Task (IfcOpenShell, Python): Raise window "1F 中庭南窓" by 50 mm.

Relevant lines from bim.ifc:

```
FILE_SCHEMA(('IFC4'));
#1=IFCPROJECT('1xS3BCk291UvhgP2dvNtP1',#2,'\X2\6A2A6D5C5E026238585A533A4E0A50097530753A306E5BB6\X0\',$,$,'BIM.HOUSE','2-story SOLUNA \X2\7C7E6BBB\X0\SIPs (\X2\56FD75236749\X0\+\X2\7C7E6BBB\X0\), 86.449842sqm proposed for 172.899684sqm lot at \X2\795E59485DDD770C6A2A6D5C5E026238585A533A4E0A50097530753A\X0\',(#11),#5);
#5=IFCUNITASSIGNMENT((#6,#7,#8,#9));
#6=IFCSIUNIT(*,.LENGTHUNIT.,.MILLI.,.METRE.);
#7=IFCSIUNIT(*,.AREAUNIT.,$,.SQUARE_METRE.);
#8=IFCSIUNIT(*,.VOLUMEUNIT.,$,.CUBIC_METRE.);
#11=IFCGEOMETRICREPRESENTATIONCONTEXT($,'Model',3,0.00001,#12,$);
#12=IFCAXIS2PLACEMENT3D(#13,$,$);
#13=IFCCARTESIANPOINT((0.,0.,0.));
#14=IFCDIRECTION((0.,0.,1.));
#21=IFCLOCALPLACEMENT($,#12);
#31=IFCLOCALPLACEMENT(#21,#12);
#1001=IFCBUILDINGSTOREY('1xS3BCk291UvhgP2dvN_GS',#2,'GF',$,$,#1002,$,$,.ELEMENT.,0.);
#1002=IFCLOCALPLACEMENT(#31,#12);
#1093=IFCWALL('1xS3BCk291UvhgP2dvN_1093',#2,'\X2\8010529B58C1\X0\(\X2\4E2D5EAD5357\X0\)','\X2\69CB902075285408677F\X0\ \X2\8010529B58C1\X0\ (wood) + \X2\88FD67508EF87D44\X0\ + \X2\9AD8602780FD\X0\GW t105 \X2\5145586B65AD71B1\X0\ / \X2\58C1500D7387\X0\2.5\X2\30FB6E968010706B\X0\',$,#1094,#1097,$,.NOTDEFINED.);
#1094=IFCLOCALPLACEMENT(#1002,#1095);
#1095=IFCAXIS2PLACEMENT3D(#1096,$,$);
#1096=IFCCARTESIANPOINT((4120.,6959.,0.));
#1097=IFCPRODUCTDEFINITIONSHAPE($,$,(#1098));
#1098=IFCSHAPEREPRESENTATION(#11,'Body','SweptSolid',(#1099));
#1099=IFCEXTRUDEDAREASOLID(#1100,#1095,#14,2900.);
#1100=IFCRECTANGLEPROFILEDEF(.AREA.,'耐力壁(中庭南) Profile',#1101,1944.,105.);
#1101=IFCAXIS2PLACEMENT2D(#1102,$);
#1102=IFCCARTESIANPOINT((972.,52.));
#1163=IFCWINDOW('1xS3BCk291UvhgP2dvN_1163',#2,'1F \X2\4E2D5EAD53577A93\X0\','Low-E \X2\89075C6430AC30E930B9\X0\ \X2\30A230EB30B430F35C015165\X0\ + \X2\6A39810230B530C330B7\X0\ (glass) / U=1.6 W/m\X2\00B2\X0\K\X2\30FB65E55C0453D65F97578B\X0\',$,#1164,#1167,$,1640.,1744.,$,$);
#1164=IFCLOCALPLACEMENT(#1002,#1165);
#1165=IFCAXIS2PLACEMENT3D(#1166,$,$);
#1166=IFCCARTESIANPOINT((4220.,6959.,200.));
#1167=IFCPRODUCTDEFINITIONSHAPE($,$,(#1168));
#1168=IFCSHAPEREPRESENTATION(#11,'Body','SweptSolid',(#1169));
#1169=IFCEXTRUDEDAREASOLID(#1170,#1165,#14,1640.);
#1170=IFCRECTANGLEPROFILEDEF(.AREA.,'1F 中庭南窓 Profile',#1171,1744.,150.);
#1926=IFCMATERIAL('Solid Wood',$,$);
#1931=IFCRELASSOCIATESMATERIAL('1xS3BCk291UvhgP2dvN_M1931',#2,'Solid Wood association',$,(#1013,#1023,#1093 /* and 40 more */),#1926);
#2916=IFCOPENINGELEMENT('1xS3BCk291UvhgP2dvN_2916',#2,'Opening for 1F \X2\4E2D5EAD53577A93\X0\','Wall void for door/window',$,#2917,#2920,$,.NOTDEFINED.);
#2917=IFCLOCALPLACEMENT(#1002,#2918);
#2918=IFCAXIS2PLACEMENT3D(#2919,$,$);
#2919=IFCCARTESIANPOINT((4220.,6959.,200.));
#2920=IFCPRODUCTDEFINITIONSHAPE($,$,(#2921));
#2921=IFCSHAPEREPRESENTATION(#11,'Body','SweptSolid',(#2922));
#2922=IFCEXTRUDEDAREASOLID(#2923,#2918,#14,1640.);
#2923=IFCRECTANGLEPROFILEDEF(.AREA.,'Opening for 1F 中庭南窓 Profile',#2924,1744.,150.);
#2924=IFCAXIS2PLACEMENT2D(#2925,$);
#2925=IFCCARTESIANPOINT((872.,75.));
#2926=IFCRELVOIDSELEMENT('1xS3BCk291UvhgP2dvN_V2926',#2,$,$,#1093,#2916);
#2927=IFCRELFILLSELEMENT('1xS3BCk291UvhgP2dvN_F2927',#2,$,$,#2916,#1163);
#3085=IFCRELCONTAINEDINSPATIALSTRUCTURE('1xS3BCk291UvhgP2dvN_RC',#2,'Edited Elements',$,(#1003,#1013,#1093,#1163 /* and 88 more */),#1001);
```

```python
import numpy as np
import ifcopenshell
import ifcopenshell.api.geometry
import ifcopenshell.util.placement
import ifcopenshell.util.unit

model = ifcopenshell.open("bim.ifc")
unit_scale = ifcopenshell.util.unit.calculate_unit_scale(model)

window = model.by_guid("1xS3BCk291UvhgP2dvN_1163")
opening = window.FillsVoids[0].RelatingOpeningElement
dz = 0.05 / unit_scale

shift = np.array([0.0, 0.0, dz])
# The window is not placed relative to its opening, so move both.
for product in (opening, window):
    matrix = ifcopenshell.util.placement.get_local_placement(product.ObjectPlacement)
    matrix[:3, 3] += shift
    ifcopenshell.api.geometry.edit_object_placement(model, product=product, matrix=matrix, is_si=False)

print(f"moved by {dz * unit_scale:+.3f} m")

model.write("bim_updated.ifc")
```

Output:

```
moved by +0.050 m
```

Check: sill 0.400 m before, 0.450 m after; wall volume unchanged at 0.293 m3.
